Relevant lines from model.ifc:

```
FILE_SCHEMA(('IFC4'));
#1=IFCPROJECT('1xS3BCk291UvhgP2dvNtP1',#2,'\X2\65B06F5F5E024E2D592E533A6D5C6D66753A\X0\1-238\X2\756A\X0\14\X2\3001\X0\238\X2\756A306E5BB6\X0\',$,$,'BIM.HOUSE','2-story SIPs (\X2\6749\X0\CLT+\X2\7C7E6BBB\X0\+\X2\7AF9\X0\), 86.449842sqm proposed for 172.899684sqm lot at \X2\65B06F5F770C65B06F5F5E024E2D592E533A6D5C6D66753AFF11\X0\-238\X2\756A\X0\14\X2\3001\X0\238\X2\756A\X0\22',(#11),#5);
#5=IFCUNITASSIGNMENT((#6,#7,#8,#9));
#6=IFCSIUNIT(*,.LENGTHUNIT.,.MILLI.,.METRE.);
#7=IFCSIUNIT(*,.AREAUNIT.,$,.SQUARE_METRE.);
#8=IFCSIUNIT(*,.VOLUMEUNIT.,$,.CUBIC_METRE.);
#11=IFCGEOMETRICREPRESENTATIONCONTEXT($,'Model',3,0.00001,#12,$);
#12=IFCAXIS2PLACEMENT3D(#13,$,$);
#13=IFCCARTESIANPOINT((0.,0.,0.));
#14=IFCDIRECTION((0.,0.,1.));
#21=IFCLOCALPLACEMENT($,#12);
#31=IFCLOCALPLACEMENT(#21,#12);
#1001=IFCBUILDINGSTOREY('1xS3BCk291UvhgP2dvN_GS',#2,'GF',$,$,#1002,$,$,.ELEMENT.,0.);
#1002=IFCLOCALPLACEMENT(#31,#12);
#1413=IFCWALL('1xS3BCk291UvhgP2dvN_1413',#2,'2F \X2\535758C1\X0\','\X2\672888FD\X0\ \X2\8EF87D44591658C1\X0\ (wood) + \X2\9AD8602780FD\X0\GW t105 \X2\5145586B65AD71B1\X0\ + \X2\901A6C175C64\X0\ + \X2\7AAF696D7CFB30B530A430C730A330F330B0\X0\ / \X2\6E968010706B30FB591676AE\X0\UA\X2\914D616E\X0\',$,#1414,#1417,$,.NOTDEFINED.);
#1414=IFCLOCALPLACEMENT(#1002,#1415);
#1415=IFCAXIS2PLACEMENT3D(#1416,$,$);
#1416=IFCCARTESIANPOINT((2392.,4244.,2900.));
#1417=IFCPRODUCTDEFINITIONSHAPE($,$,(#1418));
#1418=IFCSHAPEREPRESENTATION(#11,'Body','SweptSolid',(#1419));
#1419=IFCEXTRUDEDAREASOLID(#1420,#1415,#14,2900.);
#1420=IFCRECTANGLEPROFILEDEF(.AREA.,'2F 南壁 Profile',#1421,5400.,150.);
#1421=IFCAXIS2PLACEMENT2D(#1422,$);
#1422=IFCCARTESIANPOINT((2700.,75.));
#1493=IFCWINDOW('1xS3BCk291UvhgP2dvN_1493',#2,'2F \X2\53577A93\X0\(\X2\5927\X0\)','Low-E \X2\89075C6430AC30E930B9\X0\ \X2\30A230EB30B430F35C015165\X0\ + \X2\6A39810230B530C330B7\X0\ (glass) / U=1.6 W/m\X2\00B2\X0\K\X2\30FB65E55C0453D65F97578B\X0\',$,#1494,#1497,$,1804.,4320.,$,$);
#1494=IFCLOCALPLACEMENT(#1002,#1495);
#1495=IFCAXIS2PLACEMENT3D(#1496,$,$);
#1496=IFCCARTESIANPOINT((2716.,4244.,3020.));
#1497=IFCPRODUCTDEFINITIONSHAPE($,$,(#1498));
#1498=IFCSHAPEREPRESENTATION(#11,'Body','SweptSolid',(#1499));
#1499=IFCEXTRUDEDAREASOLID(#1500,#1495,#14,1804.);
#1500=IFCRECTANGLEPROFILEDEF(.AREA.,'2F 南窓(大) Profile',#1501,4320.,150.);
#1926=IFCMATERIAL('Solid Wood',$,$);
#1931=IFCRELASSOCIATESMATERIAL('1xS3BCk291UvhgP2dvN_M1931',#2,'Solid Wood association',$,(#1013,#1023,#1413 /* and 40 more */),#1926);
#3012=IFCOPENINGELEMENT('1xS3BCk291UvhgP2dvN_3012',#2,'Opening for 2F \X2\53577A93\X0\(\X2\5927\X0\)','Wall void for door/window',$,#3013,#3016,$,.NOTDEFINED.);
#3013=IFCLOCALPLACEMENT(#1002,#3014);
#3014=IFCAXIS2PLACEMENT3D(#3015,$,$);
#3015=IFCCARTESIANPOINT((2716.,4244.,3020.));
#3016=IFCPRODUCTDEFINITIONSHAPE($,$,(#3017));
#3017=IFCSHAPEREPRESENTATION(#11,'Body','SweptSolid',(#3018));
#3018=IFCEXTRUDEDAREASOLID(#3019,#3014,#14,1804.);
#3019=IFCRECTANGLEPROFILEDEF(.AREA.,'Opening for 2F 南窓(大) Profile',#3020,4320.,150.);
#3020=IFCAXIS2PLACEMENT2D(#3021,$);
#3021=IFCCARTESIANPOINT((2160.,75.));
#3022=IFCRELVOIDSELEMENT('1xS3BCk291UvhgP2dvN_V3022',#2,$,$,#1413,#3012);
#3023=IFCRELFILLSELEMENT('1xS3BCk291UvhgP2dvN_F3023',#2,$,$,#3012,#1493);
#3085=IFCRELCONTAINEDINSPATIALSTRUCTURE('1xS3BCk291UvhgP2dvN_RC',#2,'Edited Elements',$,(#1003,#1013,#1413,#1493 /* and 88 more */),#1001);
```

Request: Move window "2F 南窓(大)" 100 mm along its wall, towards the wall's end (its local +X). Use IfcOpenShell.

```python
import ifcopenshell
import ifcopenshell.api.geometry
import ifcopenshell.util.placement
import ifcopenshell.util.unit

model = ifcopenshell.open("model.ifc")
unit_scale = ifcopenshell.util.unit.calculate_unit_scale(model)

window = model.by_id(1493)
opening = window.FillsVoids[0].RelatingOpeningElement
wall = opening.VoidsElements[0].RelatingBuildingElement

wall_matrix = ifcopenshell.util.placement.get_local_placement(wall.ObjectPlacement)
shift = wall_matrix[:3, 0] * 0.1 / unit_scale
before = ifcopenshell.util.placement.get_local_placement(window.ObjectPlacement)[:3, 3].copy()

# The window is not placed relative to its opening, so move both.
for product in (opening, window):
    matrix = ifcopenshell.util.placement.get_local_placement(product.ObjectPlacement)
    matrix[:3, 3] += shift
    ifcopenshell.api.geometry.edit_object_placement(model, product=product, matrix=matrix, is_si=False)

after = ifcopenshell.util.placement.get_local_placement(window.ObjectPlacement)[:3, 3]
print("window moved by", (after - before).round(3) + 0.0)

model.write("model-out.ifc")
```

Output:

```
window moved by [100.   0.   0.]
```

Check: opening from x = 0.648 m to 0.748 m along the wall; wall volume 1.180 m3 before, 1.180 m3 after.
